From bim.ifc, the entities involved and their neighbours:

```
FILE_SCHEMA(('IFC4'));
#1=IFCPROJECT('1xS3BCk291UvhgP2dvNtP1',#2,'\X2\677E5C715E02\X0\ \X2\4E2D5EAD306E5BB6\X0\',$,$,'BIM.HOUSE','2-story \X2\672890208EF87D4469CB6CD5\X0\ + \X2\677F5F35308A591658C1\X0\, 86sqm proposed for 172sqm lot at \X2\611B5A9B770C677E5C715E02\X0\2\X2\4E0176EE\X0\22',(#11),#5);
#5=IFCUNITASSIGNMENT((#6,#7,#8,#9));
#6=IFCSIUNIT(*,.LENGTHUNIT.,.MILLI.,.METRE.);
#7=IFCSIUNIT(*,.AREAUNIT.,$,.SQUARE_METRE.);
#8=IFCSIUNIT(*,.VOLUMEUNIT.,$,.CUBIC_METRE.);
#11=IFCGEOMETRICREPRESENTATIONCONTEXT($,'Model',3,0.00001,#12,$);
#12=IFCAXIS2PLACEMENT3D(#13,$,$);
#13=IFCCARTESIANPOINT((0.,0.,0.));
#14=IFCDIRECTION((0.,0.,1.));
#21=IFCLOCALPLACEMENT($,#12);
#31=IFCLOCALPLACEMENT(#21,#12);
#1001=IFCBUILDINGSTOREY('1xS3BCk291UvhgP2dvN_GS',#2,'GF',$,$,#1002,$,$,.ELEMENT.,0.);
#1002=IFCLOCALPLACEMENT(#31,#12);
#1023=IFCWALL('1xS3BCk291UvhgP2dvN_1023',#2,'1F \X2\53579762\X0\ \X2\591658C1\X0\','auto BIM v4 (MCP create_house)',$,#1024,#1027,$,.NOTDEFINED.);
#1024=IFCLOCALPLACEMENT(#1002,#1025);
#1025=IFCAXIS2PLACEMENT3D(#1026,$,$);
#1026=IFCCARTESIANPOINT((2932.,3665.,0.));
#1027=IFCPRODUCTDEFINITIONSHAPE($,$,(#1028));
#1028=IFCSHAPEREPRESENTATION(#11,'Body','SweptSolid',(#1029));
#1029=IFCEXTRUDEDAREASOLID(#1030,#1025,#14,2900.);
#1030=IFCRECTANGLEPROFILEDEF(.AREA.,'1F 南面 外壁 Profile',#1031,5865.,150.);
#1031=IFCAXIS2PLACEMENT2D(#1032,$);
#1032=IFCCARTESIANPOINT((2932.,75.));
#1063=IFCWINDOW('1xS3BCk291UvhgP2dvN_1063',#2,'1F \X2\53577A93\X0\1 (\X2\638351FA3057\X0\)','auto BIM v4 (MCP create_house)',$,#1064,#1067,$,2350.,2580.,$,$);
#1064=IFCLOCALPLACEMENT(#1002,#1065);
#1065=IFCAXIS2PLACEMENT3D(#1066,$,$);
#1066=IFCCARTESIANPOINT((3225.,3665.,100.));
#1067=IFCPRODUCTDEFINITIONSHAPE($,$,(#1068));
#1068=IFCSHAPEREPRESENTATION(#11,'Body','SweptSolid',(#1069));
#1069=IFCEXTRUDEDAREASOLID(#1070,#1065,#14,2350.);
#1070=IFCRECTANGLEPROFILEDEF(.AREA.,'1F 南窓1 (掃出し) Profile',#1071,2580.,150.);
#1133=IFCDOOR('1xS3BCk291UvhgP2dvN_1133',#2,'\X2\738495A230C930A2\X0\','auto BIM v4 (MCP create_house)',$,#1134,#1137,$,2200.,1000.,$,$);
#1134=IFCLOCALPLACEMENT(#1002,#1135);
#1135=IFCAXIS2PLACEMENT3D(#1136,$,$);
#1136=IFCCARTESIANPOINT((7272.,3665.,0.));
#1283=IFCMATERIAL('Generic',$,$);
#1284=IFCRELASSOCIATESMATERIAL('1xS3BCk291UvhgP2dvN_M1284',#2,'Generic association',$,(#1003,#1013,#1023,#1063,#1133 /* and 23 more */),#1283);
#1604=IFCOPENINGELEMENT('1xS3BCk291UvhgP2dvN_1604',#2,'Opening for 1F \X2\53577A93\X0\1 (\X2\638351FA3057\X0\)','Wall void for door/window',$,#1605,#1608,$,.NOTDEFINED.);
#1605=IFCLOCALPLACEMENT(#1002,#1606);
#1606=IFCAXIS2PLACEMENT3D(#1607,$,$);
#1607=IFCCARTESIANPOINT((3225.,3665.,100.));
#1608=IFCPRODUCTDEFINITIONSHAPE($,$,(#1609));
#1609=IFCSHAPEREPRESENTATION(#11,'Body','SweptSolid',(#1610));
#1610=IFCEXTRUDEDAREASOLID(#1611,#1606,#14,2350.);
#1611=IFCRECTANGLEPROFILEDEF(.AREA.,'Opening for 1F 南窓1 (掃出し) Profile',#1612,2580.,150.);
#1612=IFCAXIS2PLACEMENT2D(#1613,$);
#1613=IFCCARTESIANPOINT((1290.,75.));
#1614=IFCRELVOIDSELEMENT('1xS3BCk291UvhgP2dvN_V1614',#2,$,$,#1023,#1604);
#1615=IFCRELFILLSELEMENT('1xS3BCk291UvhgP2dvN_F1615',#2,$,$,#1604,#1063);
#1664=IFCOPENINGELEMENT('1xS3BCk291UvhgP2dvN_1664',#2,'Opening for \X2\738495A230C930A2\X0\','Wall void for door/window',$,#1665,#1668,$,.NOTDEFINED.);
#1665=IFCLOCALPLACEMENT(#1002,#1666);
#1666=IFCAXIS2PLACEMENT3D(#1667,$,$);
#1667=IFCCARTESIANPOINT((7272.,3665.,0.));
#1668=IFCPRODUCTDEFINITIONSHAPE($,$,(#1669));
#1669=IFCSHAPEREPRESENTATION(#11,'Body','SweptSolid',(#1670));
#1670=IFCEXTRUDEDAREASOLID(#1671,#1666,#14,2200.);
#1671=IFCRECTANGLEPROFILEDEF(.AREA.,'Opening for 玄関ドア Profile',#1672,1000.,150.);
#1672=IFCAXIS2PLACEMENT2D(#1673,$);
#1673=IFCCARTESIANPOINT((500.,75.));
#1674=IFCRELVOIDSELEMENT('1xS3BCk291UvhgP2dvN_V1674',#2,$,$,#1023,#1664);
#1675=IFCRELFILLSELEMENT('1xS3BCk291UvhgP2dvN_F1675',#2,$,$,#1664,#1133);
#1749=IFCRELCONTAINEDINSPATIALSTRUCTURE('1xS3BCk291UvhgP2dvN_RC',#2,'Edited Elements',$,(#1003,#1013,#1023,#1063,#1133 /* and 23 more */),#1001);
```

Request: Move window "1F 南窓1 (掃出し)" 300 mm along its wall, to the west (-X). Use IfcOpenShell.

```python
import ifcopenshell
import ifcopenshell.api.geometry
import ifcopenshell.util.placement

model = ifcopenshell.open("bim.ifc")

window = model.by_guid("1xS3BCk291UvhgP2dvN_1063")
opening = window.FillsVoids[0].RelatingOpeningElement
wall = opening.VoidsElements[0].RelatingBuildingElement

wall_matrix = ifcopenshell.util.placement.get_local_placement(wall.ObjectPlacement)
shift = wall_matrix[:3, 0] * -300.0
before = ifcopenshell.util.placement.get_local_placement(window.ObjectPlacement)[:3, 3].copy()

# The window is not placed relative to its opening, so move both.
for product in (opening, window):
    matrix = ifcopenshell.util.placement.get_local_placement(product.ObjectPlacement)
    matrix[:3, 3] += shift
    ifcopenshell.api.geometry.edit_object_placement(model, product=product, matrix=matrix, is_si=False)

after = ifcopenshell.util.placement.get_local_placement(window.ObjectPlacement)[:3, 3]
print("window moved by", (after - before).round(3) + 0.0)

model.write("bim_edited.ifc")
```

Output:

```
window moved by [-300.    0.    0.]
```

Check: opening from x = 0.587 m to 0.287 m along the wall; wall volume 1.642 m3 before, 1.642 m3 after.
